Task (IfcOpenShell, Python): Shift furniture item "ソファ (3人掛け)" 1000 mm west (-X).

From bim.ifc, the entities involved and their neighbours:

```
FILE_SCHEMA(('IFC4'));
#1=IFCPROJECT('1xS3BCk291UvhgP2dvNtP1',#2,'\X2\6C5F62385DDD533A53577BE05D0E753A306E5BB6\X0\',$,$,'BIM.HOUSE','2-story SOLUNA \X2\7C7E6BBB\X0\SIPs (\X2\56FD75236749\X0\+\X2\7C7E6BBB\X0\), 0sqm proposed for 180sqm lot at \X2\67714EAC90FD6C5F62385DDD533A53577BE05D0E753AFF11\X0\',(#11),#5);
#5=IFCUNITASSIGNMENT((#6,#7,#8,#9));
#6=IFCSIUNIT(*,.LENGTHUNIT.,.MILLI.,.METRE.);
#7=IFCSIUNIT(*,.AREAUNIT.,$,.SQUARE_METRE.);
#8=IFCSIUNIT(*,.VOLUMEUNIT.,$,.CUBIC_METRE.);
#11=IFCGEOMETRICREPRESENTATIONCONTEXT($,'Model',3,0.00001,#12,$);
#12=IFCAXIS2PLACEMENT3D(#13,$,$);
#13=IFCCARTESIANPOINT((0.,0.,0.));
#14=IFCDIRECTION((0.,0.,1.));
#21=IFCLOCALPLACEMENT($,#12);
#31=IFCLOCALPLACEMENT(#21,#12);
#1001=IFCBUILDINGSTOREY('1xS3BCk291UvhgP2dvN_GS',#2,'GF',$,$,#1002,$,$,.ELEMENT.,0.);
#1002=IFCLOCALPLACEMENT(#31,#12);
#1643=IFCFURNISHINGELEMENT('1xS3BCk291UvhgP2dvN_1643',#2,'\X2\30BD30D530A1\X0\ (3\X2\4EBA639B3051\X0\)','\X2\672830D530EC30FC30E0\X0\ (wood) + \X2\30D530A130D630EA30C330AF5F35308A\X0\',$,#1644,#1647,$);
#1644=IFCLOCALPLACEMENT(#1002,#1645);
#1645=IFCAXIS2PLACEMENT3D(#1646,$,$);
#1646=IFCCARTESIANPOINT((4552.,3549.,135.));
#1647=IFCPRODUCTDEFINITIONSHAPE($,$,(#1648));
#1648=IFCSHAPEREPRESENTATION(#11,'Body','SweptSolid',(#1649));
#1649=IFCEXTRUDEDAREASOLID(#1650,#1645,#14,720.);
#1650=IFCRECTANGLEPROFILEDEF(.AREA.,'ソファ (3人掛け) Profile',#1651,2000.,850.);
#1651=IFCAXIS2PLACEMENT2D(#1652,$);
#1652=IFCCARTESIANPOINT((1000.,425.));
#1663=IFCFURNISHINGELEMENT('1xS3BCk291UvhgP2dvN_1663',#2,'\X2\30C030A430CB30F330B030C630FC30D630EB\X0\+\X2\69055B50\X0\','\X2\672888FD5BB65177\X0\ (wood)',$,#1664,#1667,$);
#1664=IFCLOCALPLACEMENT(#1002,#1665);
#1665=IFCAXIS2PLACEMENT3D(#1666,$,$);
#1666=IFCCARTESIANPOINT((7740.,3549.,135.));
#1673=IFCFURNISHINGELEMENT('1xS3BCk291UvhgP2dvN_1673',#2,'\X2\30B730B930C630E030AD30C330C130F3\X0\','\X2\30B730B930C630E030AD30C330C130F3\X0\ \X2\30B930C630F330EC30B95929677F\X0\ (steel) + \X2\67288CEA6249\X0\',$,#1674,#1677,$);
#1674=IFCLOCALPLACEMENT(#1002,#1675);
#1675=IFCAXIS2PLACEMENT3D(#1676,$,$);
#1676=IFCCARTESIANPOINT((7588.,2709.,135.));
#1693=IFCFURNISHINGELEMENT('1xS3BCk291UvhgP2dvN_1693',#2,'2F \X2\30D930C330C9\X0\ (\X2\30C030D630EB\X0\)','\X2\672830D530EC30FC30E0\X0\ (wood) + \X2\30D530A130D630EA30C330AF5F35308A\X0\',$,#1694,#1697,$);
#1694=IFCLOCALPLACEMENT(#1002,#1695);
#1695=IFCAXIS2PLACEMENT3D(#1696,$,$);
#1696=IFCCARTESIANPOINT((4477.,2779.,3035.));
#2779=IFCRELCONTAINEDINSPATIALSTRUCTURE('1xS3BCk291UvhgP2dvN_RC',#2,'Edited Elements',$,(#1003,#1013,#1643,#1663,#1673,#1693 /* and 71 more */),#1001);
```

```python
import ifcopenshell
import ifcopenshell.api.geometry
import ifcopenshell.util.placement
import ifcopenshell.util.unit

model = ifcopenshell.open("bim.ifc")
unit_scale = ifcopenshell.util.unit.calculate_unit_scale(model)

item = model.by_guid("1xS3BCk291UvhgP2dvN_1643")
matrix = ifcopenshell.util.placement.get_local_placement(item.ObjectPlacement)
matrix[0, 3] -= 1 / unit_scale
ifcopenshell.api.geometry.edit_object_placement(model, product=item, matrix=matrix, is_si=False)

print(ifcopenshell.util.placement.get_local_placement(item.ObjectPlacement).round(3) + 0.0)

model.write("bim-out.ifc")
```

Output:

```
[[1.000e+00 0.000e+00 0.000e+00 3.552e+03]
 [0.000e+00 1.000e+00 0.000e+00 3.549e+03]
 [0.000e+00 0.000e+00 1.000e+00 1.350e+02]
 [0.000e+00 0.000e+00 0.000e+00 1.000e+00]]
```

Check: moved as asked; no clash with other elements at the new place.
